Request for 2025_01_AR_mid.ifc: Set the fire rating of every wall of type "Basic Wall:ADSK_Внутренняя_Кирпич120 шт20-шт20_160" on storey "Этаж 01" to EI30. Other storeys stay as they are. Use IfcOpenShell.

First a look at what the model holds.

```python
import ifcopenshell
import ifcopenshell.util.element

model = ifcopenshell.open("2025_01_AR_mid.ifc")
print(model.schema)
storey = next(s for s in model.by_type("IfcBuildingStorey") if s.Name == "Этаж 01")
walls = [e for e in ifcopenshell.util.element.get_decomposition(storey) if e.is_a("IfcWall")]
seen = {}
for e in walls:
    element_type = ifcopenshell.util.element.get_type(e)
    key = (element_type.Name if element_type != e and element_type else None, ifcopenshell.util.element.get_pset(e, "Pset_WallCommon", "FireRating"))
    seen[key] = seen.get(key, 0) + 1
for (name, value), count in sorted(seen.items(), key=str):
    print(count, "x", name, "|", value)
```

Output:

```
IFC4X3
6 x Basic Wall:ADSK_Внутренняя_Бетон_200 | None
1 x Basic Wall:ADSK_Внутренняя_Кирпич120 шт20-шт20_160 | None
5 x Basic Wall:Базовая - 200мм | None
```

```python
import ifcopenshell
import ifcopenshell.api.pset
import ifcopenshell.util.element

model = ifcopenshell.open("2025_01_AR_mid.ifc")

storey = next(s for s in model.by_type("IfcBuildingStorey") if s.Name == "Этаж 01")
walls = [e for e in ifcopenshell.util.element.get_decomposition(storey) if e.is_a("IfcWall")]

count = 0
for e in walls:
    element_type = ifcopenshell.util.element.get_type(e)
    if element_type in (None, e) or element_type.Name != "Basic Wall:ADSK_Внутренняя_Кирпич120 шт20-шт20_160":
        continue
    # add_pset returns the element's existing set when there is one.
    pset = ifcopenshell.api.pset.add_pset(model, product=e, name="Pset_WallCommon")
    ifcopenshell.api.pset.edit_pset(model, pset=pset, properties={"FireRating": "EI30"})
    count += 1

print(count, "walls updated")

model.write("2025_01_AR_mid-out.ifc")
```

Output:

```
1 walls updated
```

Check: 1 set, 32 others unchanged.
